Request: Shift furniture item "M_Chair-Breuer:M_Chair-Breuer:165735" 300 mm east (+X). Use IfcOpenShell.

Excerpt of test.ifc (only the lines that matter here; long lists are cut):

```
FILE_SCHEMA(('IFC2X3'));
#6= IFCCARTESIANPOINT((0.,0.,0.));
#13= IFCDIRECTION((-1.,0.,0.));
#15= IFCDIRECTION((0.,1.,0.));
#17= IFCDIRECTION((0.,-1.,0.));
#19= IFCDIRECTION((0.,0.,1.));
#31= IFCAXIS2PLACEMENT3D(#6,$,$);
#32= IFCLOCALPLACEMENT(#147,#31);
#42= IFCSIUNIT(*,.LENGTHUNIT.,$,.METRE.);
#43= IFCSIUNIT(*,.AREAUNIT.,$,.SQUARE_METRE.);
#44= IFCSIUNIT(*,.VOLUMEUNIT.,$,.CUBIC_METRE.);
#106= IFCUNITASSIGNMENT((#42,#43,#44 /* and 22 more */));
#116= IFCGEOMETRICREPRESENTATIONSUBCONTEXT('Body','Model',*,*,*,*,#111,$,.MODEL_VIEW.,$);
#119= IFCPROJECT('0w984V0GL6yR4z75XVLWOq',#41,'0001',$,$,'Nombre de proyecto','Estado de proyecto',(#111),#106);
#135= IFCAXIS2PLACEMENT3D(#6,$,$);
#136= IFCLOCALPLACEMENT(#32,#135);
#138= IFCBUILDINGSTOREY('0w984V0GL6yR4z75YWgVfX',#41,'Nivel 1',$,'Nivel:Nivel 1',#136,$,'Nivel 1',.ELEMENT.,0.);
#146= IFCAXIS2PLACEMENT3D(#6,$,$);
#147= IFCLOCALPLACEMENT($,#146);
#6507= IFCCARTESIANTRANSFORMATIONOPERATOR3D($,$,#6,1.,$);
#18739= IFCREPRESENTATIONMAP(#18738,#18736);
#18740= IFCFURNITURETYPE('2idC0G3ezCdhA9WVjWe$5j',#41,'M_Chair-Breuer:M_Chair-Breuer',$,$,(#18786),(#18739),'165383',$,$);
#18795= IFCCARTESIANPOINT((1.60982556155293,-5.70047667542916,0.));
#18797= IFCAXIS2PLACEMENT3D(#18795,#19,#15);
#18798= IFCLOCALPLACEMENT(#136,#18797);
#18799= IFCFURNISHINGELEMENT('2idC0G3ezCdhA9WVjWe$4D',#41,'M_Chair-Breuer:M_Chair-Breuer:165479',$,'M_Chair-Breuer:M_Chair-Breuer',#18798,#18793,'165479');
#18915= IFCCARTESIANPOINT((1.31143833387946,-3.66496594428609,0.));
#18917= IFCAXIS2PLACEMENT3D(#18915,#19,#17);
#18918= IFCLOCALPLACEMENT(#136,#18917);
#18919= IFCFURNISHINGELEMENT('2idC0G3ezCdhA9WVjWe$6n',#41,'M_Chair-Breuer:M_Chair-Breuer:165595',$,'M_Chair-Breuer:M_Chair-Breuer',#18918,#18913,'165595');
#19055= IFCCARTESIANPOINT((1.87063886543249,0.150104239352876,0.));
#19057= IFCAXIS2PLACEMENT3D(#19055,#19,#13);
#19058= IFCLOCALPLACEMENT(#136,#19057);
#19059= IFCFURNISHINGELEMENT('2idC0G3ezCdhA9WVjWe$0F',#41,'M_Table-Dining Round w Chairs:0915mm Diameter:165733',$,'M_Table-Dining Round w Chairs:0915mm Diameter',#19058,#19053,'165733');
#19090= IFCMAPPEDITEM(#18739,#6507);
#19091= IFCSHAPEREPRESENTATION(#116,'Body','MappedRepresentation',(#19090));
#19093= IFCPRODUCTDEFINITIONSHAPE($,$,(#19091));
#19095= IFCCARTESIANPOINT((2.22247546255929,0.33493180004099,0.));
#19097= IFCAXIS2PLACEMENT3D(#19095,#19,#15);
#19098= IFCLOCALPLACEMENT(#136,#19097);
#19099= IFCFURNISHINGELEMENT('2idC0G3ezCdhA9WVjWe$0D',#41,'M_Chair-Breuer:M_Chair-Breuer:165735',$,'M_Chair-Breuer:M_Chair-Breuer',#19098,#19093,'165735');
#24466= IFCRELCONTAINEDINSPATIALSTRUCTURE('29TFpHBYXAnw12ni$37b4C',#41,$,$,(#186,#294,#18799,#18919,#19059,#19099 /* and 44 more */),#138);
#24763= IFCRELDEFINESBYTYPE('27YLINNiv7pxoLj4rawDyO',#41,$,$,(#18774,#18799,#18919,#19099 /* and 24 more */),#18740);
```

```python
import ifcopenshell
import ifcopenshell.api.geometry
import ifcopenshell.util.placement
import ifcopenshell.util.unit

model = ifcopenshell.open("test.ifc")
unit_scale = ifcopenshell.util.unit.calculate_unit_scale(model)

item = model.by_id(19099)
matrix = ifcopenshell.util.placement.get_local_placement(item.ObjectPlacement)
matrix[0, 3] += 0.3 / unit_scale
ifcopenshell.api.geometry.edit_object_placement(model, product=item, matrix=matrix, is_si=False)

print(ifcopenshell.util.placement.get_local_placement(item.ObjectPlacement).round(3) + 0.0)

model.write("test_rev.ifc")
```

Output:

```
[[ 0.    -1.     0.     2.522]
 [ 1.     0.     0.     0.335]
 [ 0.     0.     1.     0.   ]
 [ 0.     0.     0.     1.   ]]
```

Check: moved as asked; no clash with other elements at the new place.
